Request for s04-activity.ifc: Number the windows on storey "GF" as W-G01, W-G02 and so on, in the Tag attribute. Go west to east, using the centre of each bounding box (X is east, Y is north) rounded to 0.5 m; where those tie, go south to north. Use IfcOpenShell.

First a look at what the model holds.

```python
import ifcopenshell
import ifcopenshell.util.element
import ifcopenshell.util.placement

model = ifcopenshell.open("s04-activity.ifc")
print(model.schema)
storey = next(s for s in model.by_type("IfcBuildingStorey") if s.Name == "GF")
windows = [e for e in ifcopenshell.util.element.get_decomposition(storey) if e.is_a("IfcWindow")]
for e in sorted(windows, key=lambda e: e.id()):
    origin = ifcopenshell.util.placement.get_local_placement(e.ObjectPlacement)[:3, 3]
    print(e.id(), e.Tag, e.Name, origin.round(2) + 0.0, sep=" | ")
```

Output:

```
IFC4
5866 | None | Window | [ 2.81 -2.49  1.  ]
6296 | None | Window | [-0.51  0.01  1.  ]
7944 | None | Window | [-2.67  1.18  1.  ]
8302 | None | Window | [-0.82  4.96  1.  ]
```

```python
import ifcopenshell
import ifcopenshell.geom
import ifcopenshell.util.element
import ifcopenshell.util.shape

model = ifcopenshell.open("s04-activity.ifc")
settings = ifcopenshell.geom.settings()
settings.set("use-world-coords", True)


def centre(element):
    shape = ifcopenshell.geom.create_shape(settings, element)
    return ifcopenshell.util.shape.get_bbox_centroid(shape.geometry)


storey = next(s for s in model.by_type("IfcBuildingStorey") if s.Name == "GF")
windows = [e for e in ifcopenshell.util.element.get_decomposition(storey) if e.is_a("IfcWindow")]

# Insertion points can sit at a corner or the storey origin, so sort by the geometry (in metres).
centres = {e: centre(e) for e in windows}
windows.sort(key=lambda e: (round(centres[e][0] / 0.5), centres[e][1]))

for i, e in enumerate(windows, start=1):
    number = f"W-G{i:02d}"
    e.Tag = number
    print(e.id(), number)

model.write("s04-activity-out.ifc")
```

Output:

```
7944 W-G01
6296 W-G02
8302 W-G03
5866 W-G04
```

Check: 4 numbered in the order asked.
